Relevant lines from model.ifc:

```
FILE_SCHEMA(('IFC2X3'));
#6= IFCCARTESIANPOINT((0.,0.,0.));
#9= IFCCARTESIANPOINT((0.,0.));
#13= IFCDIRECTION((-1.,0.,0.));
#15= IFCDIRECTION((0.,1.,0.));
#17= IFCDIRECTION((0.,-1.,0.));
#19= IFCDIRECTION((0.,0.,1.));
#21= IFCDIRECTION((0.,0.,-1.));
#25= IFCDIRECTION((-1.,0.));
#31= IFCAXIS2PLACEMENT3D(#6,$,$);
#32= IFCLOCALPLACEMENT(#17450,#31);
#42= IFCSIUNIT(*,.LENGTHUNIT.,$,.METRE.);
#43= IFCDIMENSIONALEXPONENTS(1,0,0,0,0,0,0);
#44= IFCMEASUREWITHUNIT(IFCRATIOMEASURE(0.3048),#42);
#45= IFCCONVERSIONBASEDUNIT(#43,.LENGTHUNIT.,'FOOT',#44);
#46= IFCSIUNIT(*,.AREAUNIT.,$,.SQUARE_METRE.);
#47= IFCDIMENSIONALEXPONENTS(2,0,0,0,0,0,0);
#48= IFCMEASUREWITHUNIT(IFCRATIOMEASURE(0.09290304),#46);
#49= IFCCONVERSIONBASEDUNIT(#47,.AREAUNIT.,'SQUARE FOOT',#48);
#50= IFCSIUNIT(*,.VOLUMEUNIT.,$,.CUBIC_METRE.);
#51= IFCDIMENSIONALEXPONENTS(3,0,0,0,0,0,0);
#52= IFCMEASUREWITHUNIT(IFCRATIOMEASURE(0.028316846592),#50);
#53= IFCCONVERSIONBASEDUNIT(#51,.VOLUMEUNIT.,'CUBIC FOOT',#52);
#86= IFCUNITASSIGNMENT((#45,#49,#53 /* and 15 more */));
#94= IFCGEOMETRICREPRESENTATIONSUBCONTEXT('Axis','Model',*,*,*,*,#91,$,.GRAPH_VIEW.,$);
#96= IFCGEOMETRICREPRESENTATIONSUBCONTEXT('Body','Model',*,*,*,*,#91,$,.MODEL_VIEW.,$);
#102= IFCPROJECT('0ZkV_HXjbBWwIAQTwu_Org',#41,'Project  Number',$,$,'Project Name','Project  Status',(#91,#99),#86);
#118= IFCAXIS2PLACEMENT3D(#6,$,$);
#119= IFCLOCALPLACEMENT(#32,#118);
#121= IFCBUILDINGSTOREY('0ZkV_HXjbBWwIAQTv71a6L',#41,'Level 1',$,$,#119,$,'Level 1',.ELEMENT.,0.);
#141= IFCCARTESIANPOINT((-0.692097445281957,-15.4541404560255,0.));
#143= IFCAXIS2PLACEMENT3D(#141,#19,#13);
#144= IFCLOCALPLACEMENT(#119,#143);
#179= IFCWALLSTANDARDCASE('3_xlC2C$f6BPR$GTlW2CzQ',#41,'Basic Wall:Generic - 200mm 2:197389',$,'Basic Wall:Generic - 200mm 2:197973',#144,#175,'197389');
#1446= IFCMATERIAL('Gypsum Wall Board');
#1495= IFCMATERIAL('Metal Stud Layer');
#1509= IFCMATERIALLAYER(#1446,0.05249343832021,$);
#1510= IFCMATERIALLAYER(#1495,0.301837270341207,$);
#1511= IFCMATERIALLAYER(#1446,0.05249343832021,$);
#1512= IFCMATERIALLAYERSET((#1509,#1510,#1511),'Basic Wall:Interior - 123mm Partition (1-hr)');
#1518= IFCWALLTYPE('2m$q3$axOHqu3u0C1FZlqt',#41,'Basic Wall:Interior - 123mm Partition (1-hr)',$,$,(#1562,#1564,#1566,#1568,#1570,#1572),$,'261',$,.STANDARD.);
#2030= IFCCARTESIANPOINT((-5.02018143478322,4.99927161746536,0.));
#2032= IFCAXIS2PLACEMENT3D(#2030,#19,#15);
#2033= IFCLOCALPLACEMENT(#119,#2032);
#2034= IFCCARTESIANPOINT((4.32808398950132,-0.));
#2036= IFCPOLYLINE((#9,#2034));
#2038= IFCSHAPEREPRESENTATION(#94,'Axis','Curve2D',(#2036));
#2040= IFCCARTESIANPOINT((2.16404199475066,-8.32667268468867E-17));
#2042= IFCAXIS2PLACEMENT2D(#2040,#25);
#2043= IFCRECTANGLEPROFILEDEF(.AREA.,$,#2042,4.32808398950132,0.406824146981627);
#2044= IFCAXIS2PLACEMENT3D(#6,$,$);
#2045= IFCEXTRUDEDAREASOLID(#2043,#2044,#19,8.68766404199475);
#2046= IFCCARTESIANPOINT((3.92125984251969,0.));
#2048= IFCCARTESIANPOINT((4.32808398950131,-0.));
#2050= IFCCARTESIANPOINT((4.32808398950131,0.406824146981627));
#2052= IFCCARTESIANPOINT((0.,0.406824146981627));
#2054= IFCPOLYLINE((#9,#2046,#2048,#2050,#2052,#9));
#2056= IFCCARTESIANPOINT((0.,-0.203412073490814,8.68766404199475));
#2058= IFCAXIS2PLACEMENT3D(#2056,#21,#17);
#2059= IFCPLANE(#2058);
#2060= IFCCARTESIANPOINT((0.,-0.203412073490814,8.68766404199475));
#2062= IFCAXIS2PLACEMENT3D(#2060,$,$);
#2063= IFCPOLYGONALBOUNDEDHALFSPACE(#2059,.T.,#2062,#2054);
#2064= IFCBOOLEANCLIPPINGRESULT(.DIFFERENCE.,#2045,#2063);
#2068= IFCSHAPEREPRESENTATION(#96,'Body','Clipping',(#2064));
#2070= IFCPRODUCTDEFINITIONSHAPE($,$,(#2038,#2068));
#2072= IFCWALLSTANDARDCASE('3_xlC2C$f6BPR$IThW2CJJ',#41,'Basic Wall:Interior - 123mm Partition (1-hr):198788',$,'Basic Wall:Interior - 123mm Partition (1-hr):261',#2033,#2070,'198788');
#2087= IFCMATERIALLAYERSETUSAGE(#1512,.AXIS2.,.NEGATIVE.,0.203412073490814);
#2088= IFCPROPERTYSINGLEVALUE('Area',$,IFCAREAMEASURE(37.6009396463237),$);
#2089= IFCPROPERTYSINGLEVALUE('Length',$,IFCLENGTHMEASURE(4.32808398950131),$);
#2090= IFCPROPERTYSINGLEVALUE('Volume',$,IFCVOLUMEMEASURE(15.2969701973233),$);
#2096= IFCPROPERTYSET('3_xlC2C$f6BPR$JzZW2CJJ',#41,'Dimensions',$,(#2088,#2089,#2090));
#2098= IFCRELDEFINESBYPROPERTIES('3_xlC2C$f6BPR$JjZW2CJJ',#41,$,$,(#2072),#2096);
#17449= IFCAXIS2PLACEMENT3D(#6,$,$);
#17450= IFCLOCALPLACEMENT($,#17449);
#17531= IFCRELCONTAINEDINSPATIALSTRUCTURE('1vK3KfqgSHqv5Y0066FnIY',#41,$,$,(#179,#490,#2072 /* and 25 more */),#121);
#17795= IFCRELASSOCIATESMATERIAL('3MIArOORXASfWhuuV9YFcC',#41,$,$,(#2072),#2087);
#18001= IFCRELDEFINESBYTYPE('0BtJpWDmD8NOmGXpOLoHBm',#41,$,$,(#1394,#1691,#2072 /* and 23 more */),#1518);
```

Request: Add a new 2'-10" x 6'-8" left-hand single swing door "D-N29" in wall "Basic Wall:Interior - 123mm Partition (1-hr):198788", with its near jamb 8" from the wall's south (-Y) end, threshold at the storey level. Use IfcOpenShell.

```python
import numpy as np
import ifcopenshell
import ifcopenshell.api.feature
import ifcopenshell.api.geometry
import ifcopenshell.api.pset
import ifcopenshell.api.root
import ifcopenshell.api.spatial
import ifcopenshell.api.type
import ifcopenshell.geom
import ifcopenshell.util.element
import ifcopenshell.util.placement
import ifcopenshell.util.representation
import ifcopenshell.util.shape
import ifcopenshell.util.unit

model = ifcopenshell.open("model.ifc")
unit_scale = ifcopenshell.util.unit.calculate_unit_scale(model)
area_scale = ifcopenshell.util.unit.calculate_unit_scale(model, "AREAUNIT")
volume_scale = ifcopenshell.util.unit.calculate_unit_scale(model, "VOLUMEUNIT")
settings = ifcopenshell.geom.settings()


def volume(element):
    """Net volume in cubic metres, openings subtracted."""
    shape = ifcopenshell.geom.create_shape(settings, element)
    return ifcopenshell.util.shape.get_volume(shape.geometry)


wall = model.by_guid("3_xlC2C$f6BPR$IThW2CJJ")
storey = ifcopenshell.util.element.get_container(wall, ifc_class="IfcBuildingStorey")
context = ifcopenshell.util.representation.get_context(model, "Model", "Body", "MODEL_VIEW")
before = volume(wall)

width, height, from_end, sill = 0.8636, 2.032, 0.2032, 0.0  # metres

# The wall runs along its own X axis, and the end named is its -X end.
wall_shape = ifcopenshell.geom.create_shape(settings, wall)
x, y, z = ifcopenshell.util.shape.get_vertices(wall_shape.geometry).T
start = x.min() + from_end
face, thickness = float(y.min()), float(y.max() - y.min())
wall_matrix = ifcopenshell.util.placement.get_local_placement(wall.ObjectPlacement)
level = ifcopenshell.util.placement.get_local_placement(storey.ObjectPlacement)[2, 3]


def in_wall(x, y):
    """Placement at x, y metres in the wall's axes, at sill height."""
    matrix = wall_matrix.copy()
    matrix[:, 3] = wall_matrix @ np.array([x / unit_scale, y / unit_scale, 0.0, 1.0])
    matrix[2, 3] = level + sill / unit_scale
    return matrix


# Opening: a box that overshoots both wall faces by 50 mm.
opening = ifcopenshell.api.root.create_entity(model, ifc_class="IfcOpeningElement")
box = ifcopenshell.api.geometry.add_wall_representation(
    model, context=context, length=width, height=height, thickness=thickness + 0.1
)
ifcopenshell.api.geometry.assign_representation(model, product=opening, representation=box)
ifcopenshell.api.geometry.edit_object_placement(model, product=opening, matrix=in_wall(start, face - 0.05), is_si=False)
ifcopenshell.api.feature.add_feature(model, feature=opening, element=wall)

door = ifcopenshell.api.root.create_entity(model, ifc_class="IfcDoor", name="D-N29")
door.OverallWidth, door.OverallHeight = width / unit_scale, height / unit_scale
body = ifcopenshell.api.geometry.add_door_representation(
    model,
    context=context,
    overall_width=door.OverallWidth,
    overall_height=door.OverallHeight,
    operation_type="SINGLE_SWING_LEFT",
    lining_properties={"LiningDepth": thickness / unit_scale, "ThresholdDepth": thickness / unit_scale},
)
ifcopenshell.api.geometry.assign_representation(model, product=door, representation=body)
ifcopenshell.api.spatial.assign_container(model, products=[door], relating_structure=storey)
fills = ifcopenshell.api.feature.add_filling(model, opening=opening, element=door)
fills.OwnerHistory = door.OwnerHistory  # required in IFC2X3

# IFC2X3 keeps the operation on the door style.
style = ifcopenshell.api.root.create_entity(model, ifc_class="IfcDoorStyle", name="D-N29")
style.OperationType, style.ConstructionType = "SINGLE_SWING_LEFT", "NOTDEFINED"
style.ParameterTakesPrecedence = style.Sizeable = False
ifcopenshell.api.type.assign_type(model, related_objects=[door], relating_type=style)

# The lining spans the wall, so the door starts at the wall face.
ifcopenshell.api.geometry.edit_object_placement(model, product=door, matrix=in_wall(start, face), is_si=False)

after = volume(wall)

# Update the wall's stored quantities.
pset = model.by_id(ifcopenshell.util.element.get_pset(wall, "Dimensions", should_inherit=False)["id"])
ifcopenshell.api.pset.edit_pset(model, pset=pset, properties={
    "Area": model.create_entity("IfcAreaMeasure", after / thickness / area_scale),
    "Volume": model.create_entity("IfcVolumeMeasure", after / volume_scale),
})

print(f"wall volume {before:.3f} -> {after:.3f} m3")

model.write("model_updated.ifc")
```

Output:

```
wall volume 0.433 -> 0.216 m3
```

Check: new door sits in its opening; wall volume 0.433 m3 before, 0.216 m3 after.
